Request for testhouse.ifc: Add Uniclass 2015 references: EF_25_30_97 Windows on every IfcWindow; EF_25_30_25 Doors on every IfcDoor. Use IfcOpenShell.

First a look at what the model holds.

```python
import ifcopenshell

model = ifcopenshell.open("testhouse.ifc")
print(model.schema)
print("classifications:", [c.Name for c in model.by_type("IfcClassification")])
for ifc_class in ("IfcDoor", "IfcRoof", "IfcStair", "IfcWall", "IfcWindow"):
    print(ifc_class, len(model.by_type(ifc_class)))
```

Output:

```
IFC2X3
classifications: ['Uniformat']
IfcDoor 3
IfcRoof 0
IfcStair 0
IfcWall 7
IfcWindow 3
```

```python
import ifcopenshell
import ifcopenshell.api.classification

model = ifcopenshell.open("testhouse.ifc")

# IFC2X3 requires Source and Edition and has no link from the project to the system.
system = model.create_entity("IfcClassification", Source="NBS", Edition="2015", Name="Uniclass 2015")

codes = {
    "IfcWindow": ("EF_25_30_97", "Windows"),
    "IfcDoor": ("EF_25_30_25", "Doors"),
}
for ifc_class, (code, name) in codes.items():
    products = model.by_type(ifc_class)
    ifcopenshell.api.classification.add_reference(
        model, products=products, classification=system, identification=code, name=name
    )
    print(code, len(products))

model.write("testhouse_rev.ifc")
```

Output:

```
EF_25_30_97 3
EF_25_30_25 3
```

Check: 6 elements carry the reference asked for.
